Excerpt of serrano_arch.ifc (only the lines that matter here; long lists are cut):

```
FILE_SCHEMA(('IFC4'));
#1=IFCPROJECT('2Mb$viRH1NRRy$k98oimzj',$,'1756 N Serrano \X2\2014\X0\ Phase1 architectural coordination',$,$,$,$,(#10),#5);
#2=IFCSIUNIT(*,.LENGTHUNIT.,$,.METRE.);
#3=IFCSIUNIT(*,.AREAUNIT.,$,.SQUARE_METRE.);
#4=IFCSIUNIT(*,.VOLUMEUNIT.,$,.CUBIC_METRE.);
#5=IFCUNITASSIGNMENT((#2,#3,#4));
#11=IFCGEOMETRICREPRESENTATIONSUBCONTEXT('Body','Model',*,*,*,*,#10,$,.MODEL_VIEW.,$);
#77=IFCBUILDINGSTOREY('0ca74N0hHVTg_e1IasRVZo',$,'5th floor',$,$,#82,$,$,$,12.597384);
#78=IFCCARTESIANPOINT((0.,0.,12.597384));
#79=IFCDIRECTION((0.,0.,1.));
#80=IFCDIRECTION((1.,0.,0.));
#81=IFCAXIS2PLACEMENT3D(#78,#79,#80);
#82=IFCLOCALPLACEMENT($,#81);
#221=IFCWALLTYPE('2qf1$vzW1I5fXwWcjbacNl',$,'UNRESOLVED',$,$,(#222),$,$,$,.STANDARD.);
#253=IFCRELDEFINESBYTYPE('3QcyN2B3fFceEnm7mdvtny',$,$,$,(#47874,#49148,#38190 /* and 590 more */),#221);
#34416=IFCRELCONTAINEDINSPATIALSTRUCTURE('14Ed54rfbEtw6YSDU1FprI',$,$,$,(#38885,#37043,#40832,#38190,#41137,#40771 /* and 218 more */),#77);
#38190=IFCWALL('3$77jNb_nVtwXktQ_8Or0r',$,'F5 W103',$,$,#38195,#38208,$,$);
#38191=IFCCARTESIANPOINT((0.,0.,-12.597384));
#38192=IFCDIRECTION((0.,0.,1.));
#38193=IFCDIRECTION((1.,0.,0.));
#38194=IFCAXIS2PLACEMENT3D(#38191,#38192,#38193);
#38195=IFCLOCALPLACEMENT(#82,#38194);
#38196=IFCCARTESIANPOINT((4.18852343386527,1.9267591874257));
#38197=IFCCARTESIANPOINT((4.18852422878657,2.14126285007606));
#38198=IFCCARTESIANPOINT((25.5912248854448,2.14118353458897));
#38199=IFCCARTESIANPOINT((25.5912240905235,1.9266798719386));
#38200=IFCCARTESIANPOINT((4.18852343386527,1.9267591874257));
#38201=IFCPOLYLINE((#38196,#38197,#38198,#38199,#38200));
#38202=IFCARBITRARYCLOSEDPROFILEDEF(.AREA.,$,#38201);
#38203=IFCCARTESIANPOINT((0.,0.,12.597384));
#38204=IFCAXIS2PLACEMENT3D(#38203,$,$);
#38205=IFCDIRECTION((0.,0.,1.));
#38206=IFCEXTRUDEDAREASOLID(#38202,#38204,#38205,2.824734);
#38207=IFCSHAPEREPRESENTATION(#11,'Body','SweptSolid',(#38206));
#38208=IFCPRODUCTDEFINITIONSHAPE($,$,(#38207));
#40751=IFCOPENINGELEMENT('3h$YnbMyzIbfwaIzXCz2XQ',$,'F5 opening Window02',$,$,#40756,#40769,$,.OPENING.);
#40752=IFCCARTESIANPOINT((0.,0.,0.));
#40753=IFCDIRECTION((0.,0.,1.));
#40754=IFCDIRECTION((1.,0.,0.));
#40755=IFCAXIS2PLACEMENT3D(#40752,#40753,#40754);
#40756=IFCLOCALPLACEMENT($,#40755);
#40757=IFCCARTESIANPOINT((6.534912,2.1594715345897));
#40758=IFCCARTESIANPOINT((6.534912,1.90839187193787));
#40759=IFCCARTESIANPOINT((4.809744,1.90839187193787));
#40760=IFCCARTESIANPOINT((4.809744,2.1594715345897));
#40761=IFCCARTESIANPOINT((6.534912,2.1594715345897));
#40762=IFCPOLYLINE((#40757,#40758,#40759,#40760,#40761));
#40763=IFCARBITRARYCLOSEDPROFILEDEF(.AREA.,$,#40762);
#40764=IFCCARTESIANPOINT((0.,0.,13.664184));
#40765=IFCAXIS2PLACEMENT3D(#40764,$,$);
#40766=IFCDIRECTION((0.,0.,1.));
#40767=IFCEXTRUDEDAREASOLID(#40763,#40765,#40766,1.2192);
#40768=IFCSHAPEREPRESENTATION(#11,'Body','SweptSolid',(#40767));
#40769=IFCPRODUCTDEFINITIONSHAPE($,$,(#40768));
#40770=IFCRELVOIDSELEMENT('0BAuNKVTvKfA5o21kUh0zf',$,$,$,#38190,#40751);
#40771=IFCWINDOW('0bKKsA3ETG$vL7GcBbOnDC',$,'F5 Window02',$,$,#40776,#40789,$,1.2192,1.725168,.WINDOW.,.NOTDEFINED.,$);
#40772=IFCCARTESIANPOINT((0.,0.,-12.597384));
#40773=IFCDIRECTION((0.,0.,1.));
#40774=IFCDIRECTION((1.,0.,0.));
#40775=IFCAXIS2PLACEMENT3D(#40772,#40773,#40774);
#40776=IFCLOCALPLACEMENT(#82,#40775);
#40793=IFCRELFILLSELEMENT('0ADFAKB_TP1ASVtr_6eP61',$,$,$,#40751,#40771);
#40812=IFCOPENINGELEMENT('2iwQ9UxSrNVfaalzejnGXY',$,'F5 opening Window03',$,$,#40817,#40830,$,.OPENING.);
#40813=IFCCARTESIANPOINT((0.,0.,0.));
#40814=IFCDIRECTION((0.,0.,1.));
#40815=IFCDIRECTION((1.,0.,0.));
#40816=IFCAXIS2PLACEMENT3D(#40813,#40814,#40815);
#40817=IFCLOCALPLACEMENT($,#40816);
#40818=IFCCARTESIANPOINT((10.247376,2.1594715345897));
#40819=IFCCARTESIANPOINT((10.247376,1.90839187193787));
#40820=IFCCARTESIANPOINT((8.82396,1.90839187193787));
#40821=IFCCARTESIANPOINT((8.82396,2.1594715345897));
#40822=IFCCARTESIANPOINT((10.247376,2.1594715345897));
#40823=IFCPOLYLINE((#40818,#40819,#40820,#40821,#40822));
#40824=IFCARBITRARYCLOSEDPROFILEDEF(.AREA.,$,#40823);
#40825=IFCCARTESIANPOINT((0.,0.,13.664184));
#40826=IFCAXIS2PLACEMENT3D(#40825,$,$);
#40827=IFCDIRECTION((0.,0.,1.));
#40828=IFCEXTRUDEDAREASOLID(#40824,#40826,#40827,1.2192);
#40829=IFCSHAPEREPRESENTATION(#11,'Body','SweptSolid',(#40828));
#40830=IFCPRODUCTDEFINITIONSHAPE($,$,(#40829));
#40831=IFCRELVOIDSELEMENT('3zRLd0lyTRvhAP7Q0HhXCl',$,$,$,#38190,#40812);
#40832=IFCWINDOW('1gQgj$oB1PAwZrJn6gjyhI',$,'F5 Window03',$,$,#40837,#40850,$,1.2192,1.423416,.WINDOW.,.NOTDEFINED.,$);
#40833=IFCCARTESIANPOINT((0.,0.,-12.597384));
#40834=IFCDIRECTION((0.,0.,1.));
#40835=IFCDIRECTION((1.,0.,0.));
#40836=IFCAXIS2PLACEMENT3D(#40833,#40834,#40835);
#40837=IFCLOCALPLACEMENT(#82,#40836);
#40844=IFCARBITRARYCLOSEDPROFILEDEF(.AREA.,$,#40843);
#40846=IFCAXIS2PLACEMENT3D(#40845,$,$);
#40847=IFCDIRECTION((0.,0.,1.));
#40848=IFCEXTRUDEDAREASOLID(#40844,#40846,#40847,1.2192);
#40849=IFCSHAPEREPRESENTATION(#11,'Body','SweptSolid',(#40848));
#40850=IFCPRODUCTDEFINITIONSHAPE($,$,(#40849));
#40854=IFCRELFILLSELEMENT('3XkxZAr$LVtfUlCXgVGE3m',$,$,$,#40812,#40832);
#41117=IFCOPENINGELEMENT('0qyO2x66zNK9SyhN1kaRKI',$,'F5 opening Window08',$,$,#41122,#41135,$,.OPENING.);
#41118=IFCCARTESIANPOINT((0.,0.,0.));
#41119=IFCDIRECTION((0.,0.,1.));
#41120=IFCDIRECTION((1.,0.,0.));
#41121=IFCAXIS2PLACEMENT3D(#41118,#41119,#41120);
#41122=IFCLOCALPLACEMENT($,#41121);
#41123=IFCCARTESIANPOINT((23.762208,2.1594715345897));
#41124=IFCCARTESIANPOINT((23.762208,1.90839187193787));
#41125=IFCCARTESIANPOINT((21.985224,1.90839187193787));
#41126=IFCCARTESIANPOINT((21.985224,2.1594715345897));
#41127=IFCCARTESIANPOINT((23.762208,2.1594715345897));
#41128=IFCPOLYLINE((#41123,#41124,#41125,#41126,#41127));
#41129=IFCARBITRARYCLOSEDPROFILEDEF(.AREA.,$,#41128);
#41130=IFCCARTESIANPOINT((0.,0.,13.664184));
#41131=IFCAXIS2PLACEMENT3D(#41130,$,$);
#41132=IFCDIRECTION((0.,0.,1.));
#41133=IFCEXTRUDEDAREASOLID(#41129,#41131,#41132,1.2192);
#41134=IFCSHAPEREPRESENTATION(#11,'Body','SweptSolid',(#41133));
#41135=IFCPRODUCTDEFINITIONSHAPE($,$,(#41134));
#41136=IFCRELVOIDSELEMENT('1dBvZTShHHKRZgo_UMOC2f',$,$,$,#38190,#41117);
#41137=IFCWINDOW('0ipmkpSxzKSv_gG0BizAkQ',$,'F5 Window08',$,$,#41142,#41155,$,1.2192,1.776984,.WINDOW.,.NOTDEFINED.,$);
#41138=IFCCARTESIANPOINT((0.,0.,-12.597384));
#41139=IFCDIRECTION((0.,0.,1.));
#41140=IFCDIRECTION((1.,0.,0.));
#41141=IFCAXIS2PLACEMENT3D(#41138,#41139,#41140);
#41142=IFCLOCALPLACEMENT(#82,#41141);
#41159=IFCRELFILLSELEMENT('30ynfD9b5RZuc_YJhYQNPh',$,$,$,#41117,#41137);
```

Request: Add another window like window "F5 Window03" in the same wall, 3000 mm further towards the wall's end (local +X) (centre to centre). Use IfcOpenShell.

```python
import ifcopenshell
import ifcopenshell.api.feature
import ifcopenshell.api.geometry
import ifcopenshell.api.root
import ifcopenshell.geom
import ifcopenshell.util.element
import ifcopenshell.util.placement
import ifcopenshell.util.shape

model = ifcopenshell.open("serrano_arch.ifc")
settings = ifcopenshell.geom.settings()


def volume(element):
    """Net volume in cubic metres, openings subtracted."""
    shape = ifcopenshell.geom.create_shape(settings, element)
    return ifcopenshell.util.shape.get_volume(shape.geometry)


window = model.by_guid("1gQgj$oB1PAwZrJn6gjyhI")
opening = window.FillsVoids[0].RelatingOpeningElement
wall = opening.VoidsElements[0].RelatingBuildingElement
before = volume(wall)
shift = ifcopenshell.util.placement.get_local_placement(wall.ObjectPlacement)[:3, 0] * 3.0

# copy_class copies the void relationship, type, container and properties, but no geometry.
new_opening = ifcopenshell.api.root.copy_class(model, product=opening)
new_opening.Representation = ifcopenshell.util.element.copy_deep(
    model, opening.Representation, exclude=["IfcGeometricRepresentationContext", "IfcRepresentationMap"]
)
new_window = ifcopenshell.api.root.copy_class(model, product=window)
new_window.Representation = ifcopenshell.util.element.copy_deep(
    model, window.Representation, exclude=["IfcGeometricRepresentationContext", "IfcRepresentationMap"]
)
ifcopenshell.api.feature.add_filling(model, opening=new_opening, element=new_window)

for old, new in ((opening, new_opening), (window, new_window)):
    matrix = ifcopenshell.util.placement.get_local_placement(old.ObjectPlacement)
    matrix[:3, 3] += shift
    ifcopenshell.api.geometry.edit_object_placement(model, product=new, matrix=matrix, is_si=False)

after = volume(wall)

print(f"wall volume {before:.3f} -> {after:.3f} m3")

model.write("serrano_arch_updated.ifc")
```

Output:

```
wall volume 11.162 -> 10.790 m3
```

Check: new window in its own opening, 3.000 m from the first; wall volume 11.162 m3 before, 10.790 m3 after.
